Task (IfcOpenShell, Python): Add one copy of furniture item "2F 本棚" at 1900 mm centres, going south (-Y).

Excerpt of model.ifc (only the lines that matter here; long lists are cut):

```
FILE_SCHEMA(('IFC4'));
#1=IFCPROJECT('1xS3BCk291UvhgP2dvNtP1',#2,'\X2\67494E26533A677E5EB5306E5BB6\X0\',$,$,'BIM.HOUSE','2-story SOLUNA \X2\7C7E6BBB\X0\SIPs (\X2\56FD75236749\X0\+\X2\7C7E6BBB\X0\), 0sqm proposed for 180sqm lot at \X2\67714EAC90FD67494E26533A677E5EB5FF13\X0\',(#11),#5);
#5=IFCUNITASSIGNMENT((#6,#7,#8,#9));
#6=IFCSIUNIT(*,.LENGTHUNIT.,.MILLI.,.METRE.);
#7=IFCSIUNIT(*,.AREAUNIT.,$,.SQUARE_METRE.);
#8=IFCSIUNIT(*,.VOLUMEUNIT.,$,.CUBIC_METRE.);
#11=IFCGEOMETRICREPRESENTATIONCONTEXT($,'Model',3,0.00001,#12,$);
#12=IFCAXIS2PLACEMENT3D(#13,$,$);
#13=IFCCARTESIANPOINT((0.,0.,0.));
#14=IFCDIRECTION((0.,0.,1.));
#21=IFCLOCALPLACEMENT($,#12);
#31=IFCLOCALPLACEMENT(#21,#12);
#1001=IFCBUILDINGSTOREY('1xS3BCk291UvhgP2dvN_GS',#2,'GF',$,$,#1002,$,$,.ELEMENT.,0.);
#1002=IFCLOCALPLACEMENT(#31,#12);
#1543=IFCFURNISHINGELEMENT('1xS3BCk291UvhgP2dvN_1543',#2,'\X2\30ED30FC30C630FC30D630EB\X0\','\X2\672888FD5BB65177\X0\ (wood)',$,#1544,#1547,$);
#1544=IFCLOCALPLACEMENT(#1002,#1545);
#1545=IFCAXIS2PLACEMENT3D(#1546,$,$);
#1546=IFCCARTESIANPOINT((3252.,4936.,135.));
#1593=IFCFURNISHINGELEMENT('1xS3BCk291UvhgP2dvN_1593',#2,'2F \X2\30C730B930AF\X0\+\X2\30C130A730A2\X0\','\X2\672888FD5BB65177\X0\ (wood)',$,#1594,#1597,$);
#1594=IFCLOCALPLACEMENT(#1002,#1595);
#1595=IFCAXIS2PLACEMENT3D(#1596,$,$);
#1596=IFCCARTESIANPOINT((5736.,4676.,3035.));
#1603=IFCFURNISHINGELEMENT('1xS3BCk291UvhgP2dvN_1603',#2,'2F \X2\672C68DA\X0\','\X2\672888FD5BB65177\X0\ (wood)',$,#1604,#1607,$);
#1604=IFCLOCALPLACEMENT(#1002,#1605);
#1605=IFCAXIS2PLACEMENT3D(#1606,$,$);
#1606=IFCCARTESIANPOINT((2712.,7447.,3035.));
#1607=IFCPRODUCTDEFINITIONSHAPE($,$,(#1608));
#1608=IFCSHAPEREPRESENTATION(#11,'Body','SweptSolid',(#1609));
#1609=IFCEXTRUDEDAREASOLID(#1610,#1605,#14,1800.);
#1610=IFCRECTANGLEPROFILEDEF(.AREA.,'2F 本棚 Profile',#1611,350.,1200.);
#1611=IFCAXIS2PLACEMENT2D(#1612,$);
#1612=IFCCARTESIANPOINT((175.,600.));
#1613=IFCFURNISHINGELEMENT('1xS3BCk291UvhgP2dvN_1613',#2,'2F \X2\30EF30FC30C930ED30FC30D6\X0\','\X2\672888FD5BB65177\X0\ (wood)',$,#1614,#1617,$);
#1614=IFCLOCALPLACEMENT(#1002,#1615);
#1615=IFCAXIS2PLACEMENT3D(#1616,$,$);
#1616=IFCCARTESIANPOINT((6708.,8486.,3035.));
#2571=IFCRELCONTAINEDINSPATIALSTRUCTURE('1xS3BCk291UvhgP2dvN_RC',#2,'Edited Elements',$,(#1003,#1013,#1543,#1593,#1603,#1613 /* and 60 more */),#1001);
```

```python
import numpy as np
import ifcopenshell
import ifcopenshell.api.geometry
import ifcopenshell.api.root
import ifcopenshell.util.element
import ifcopenshell.util.placement

model = ifcopenshell.open("model.ifc")


def reuse_history(source, copy):
    """copy_class also copies each property set's owner history, people and application; keep the originals."""
    for rel in copy.IsDefinedBy:
        if rel.is_a("IfcRelDefinesByProperties") and (history := rel.RelatingPropertyDefinition.OwnerHistory):
            rel.RelatingPropertyDefinition.OwnerHistory = source.OwnerHistory
            ifcopenshell.util.element.remove_deep2(model, history)


source = model.by_guid("1xS3BCk291UvhgP2dvN_1603")
base = ifcopenshell.util.placement.get_local_placement(source.ObjectPlacement)
step = np.array([0.0, -1.0, 0.0]) * 1900.0

for i in range(1, 2):
    copy = ifcopenshell.api.root.copy_class(model, product=source)
    copy.Representation = ifcopenshell.util.element.copy_deep(
        model, source.Representation, exclude=["IfcGeometricRepresentationContext", "IfcRepresentationMap"]
    )
    reuse_history(source, copy)
    matrix = base.copy()
    matrix[:3, 3] += i * step
    print("added at", matrix[:3, 3].round(3) + 0.0)
    ifcopenshell.api.geometry.edit_object_placement(model, product=copy, matrix=matrix, is_si=False)

model.write("model_edited.ifc")
```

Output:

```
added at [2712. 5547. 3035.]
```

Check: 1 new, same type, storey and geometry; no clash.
